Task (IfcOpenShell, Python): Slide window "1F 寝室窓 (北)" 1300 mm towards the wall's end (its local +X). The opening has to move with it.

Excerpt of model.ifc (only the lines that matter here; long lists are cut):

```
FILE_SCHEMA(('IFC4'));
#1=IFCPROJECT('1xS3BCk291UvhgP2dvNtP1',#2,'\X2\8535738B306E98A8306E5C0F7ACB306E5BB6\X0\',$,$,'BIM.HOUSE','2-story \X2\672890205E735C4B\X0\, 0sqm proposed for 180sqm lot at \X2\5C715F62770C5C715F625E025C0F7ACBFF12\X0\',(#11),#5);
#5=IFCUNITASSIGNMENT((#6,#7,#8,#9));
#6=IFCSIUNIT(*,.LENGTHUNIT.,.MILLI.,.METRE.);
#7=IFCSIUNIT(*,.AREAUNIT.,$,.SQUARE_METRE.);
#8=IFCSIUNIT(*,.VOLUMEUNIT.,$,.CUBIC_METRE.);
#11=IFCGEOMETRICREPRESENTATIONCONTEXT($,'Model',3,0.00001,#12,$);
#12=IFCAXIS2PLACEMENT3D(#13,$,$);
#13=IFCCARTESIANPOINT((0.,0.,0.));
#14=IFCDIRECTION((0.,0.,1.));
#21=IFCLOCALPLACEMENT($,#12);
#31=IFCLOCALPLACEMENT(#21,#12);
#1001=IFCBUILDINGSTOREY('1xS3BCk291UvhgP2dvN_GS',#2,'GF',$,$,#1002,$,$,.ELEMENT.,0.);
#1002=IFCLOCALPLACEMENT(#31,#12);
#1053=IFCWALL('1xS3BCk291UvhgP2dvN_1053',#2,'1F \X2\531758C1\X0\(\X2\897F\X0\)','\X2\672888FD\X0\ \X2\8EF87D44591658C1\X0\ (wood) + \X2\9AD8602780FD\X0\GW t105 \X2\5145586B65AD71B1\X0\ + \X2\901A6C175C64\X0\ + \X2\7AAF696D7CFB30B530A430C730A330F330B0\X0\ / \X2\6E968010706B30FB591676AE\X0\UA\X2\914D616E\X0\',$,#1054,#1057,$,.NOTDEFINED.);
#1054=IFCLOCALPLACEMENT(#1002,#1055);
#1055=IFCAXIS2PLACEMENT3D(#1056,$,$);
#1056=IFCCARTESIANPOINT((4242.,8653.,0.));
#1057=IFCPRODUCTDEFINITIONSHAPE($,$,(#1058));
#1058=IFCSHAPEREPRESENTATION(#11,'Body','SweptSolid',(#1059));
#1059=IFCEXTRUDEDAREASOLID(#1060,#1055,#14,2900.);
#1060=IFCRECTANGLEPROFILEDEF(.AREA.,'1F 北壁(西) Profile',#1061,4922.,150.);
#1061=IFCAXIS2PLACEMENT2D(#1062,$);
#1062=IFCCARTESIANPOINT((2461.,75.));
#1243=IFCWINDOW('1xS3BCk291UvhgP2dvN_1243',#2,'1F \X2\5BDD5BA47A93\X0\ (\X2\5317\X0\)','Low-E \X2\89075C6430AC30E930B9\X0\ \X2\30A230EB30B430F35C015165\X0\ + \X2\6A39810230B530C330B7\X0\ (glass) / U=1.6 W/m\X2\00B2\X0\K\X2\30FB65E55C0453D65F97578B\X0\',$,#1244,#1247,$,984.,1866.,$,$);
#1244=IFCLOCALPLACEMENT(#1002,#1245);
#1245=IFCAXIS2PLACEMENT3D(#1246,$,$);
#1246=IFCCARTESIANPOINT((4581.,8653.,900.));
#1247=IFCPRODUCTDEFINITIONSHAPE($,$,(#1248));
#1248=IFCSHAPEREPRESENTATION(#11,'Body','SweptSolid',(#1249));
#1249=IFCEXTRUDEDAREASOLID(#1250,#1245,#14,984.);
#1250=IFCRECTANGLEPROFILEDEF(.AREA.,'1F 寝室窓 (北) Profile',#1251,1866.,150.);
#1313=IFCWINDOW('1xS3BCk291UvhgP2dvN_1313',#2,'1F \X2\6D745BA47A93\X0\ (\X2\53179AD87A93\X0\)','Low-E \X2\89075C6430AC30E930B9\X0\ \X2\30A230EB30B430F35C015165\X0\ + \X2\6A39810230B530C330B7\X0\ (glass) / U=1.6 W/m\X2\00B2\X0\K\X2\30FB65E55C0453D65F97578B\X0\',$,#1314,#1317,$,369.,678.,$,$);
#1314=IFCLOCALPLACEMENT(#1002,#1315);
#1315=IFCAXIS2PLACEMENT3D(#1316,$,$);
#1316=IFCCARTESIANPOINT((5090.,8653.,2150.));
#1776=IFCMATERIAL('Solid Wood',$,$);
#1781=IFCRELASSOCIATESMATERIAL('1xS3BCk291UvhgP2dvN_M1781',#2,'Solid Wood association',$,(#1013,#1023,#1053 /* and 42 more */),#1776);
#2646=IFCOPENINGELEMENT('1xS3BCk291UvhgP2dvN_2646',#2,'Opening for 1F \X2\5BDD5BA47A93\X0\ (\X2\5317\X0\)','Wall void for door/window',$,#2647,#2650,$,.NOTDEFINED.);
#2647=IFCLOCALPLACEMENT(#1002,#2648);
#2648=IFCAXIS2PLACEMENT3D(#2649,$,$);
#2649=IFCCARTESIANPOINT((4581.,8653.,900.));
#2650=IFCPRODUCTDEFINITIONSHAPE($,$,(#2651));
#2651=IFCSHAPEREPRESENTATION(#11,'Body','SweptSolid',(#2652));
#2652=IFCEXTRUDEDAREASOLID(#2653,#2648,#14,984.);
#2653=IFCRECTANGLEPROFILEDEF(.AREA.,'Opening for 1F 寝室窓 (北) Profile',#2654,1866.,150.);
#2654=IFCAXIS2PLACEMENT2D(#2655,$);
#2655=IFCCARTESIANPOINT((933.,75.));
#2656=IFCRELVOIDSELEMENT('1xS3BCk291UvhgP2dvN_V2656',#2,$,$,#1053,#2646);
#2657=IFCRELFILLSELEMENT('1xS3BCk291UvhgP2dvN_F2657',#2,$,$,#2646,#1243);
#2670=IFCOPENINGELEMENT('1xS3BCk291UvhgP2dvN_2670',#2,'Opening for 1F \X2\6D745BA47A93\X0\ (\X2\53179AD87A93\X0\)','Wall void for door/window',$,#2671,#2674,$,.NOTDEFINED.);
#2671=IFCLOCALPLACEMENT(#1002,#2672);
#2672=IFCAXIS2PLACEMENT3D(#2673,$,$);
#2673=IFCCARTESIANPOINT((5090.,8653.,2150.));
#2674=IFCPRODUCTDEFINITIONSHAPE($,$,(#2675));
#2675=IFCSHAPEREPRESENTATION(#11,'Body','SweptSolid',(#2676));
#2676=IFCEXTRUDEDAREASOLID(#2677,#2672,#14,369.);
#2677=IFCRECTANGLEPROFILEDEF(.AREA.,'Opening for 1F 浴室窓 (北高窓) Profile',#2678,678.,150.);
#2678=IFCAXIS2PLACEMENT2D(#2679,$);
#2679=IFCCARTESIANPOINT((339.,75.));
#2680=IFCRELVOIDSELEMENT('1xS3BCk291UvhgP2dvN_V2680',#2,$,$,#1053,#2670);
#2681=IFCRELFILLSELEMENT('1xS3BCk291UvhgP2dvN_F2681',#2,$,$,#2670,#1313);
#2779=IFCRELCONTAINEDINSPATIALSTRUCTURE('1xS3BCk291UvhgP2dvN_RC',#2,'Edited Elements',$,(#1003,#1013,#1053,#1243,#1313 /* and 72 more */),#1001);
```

```python
import ifcopenshell
import ifcopenshell.api.geometry
import ifcopenshell.util.placement
import ifcopenshell.util.unit

model = ifcopenshell.open("model.ifc")
unit_scale = ifcopenshell.util.unit.calculate_unit_scale(model)

window = model.by_guid("1xS3BCk291UvhgP2dvN_1243")
opening = window.FillsVoids[0].RelatingOpeningElement
wall = opening.VoidsElements[0].RelatingBuildingElement

wall_matrix = ifcopenshell.util.placement.get_local_placement(wall.ObjectPlacement)
shift = wall_matrix[:3, 0] * 1.3 / unit_scale
before = ifcopenshell.util.placement.get_local_placement(window.ObjectPlacement)[:3, 3].copy()

# The window is not placed relative to its opening, so move both.
for product in (opening, window):
    matrix = ifcopenshell.util.placement.get_local_placement(product.ObjectPlacement)
    matrix[:3, 3] += shift
    ifcopenshell.api.geometry.edit_object_placement(model, product=product, matrix=matrix, is_si=False)

after = ifcopenshell.util.placement.get_local_placement(window.ObjectPlacement)[:3, 3]
print("window moved by", (after - before).round(3) + 0.0)

model.write("model-out.ifc")
```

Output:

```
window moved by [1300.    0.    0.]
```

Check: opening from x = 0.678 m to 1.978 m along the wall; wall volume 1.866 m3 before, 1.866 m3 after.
